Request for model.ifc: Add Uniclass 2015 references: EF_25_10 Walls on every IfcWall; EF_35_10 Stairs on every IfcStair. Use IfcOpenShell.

First a look at what the model holds.

```python
import ifcopenshell

model = ifcopenshell.open("model.ifc")
print(model.schema)
print("classifications:", [c.Name for c in model.by_type("IfcClassification")])
for ifc_class in ("IfcDoor", "IfcRoof", "IfcStair", "IfcWall", "IfcWindow"):
    print(ifc_class, len(model.by_type(ifc_class)))
```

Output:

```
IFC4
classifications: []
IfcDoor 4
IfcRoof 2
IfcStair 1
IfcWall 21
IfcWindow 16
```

```python
import ifcopenshell
import ifcopenshell.api.classification

model = ifcopenshell.open("model.ifc")

system = ifcopenshell.api.classification.add_classification(model, classification="Uniclass 2015")

codes = {
    "IfcWall": ("EF_25_10", "Walls"),
    "IfcStair": ("EF_35_10", "Stairs"),
}
for ifc_class, (code, name) in codes.items():
    products = model.by_type(ifc_class)
    ifcopenshell.api.classification.add_reference(
        model, products=products, classification=system, identification=code, name=name
    )
    print(code, len(products))

model.write("model_updated.ifc")
```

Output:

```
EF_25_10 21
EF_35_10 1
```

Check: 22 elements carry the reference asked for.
